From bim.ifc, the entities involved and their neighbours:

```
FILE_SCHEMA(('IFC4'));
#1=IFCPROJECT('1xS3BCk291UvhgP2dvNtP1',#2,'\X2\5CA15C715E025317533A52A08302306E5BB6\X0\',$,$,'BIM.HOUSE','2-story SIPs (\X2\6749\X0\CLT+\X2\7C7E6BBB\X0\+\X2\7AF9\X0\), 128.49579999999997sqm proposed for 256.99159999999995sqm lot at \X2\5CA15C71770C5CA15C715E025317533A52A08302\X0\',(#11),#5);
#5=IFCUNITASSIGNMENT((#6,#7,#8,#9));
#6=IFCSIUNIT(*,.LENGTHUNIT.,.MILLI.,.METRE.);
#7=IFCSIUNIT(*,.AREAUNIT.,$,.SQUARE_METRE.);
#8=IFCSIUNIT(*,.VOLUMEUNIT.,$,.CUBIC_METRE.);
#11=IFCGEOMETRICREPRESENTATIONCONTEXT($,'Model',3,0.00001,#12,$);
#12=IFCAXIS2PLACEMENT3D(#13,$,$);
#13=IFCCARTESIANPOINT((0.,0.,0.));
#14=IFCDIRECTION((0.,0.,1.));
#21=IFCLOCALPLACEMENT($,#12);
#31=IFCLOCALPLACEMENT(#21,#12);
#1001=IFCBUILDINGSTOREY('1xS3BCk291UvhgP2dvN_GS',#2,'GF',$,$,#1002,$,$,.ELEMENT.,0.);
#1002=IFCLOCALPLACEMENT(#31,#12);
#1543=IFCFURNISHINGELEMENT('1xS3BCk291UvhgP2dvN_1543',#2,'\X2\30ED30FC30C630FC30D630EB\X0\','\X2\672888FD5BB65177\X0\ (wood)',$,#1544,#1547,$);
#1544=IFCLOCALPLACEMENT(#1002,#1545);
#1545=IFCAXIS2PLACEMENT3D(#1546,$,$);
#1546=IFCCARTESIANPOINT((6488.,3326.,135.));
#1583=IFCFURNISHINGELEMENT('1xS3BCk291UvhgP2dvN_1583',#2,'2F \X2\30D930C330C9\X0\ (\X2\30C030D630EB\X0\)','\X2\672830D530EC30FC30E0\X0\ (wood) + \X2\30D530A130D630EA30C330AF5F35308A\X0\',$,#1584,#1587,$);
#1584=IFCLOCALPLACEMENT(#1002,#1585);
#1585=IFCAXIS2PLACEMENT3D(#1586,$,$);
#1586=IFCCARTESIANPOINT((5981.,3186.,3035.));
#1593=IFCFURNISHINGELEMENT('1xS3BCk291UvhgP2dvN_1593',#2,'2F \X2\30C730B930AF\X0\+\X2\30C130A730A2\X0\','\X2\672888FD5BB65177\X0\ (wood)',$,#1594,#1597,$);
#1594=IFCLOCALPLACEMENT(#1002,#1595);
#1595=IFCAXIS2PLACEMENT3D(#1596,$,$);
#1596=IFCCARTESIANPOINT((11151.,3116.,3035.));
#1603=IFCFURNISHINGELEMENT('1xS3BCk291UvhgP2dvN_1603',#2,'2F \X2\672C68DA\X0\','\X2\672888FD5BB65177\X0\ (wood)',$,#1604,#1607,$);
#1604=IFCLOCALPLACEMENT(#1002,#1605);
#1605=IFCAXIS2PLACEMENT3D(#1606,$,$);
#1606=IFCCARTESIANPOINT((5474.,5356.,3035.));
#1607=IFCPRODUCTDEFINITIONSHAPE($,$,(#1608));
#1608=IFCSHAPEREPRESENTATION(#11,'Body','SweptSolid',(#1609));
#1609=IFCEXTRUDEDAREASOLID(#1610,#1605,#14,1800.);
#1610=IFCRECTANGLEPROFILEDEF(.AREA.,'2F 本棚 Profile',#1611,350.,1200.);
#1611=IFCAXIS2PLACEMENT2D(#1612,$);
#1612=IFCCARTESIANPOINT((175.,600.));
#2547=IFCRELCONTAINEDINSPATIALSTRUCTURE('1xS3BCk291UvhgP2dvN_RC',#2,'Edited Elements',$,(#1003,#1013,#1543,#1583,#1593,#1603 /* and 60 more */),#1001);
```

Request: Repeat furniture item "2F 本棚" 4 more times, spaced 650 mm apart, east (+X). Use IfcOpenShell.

```python
import numpy as np
import ifcopenshell
import ifcopenshell.api.geometry
import ifcopenshell.api.root
import ifcopenshell.util.element
import ifcopenshell.util.placement
import ifcopenshell.util.unit

model = ifcopenshell.open("bim.ifc")
unit_scale = ifcopenshell.util.unit.calculate_unit_scale(model)


def reuse_history(source, copy):
    """copy_class also copies each property set's owner history, people and application; keep the originals."""
    for rel in copy.IsDefinedBy:
        if rel.is_a("IfcRelDefinesByProperties") and (history := rel.RelatingPropertyDefinition.OwnerHistory):
            rel.RelatingPropertyDefinition.OwnerHistory = source.OwnerHistory
            ifcopenshell.util.element.remove_deep2(model, history)


source = model.by_guid("1xS3BCk291UvhgP2dvN_1603")
base = ifcopenshell.util.placement.get_local_placement(source.ObjectPlacement)
step = np.array([1.0, 0.0, 0.0]) * 0.65 / unit_scale

for i in range(1, 5):
    copy = ifcopenshell.api.root.copy_class(model, product=source)
    copy.Representation = ifcopenshell.util.element.copy_deep(
        model, source.Representation, exclude=["IfcGeometricRepresentationContext", "IfcRepresentationMap"]
    )
    reuse_history(source, copy)
    matrix = base.copy()
    matrix[:3, 3] += i * step
    print("added at", matrix[:3, 3].round(3) + 0.0)
    ifcopenshell.api.geometry.edit_object_placement(model, product=copy, matrix=matrix, is_si=False)

model.write("bim-out.ifc")
```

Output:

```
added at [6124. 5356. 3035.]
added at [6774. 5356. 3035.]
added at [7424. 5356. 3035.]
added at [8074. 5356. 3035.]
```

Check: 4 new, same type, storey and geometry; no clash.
